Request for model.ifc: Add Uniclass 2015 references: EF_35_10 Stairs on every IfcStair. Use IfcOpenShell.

First a look at what the model holds.

```python
import ifcopenshell

model = ifcopenshell.open("model.ifc")
print(model.schema)
print("classifications:", [c.Name for c in model.by_type("IfcClassification")])
for ifc_class in ("IfcDoor", "IfcRoof", "IfcStair", "IfcWall", "IfcWindow"):
    print(ifc_class, len(model.by_type(ifc_class)))
```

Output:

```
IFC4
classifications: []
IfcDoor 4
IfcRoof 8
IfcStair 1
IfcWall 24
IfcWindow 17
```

```python
import ifcopenshell
import ifcopenshell.api.classification

model = ifcopenshell.open("model.ifc")

system = ifcopenshell.api.classification.add_classification(model, classification="Uniclass 2015")

codes = {
    "IfcStair": ("EF_35_10", "Stairs"),
}
for ifc_class, (code, name) in codes.items():
    products = model.by_type(ifc_class)
    ifcopenshell.api.classification.add_reference(
        model, products=products, classification=system, identification=code, name=name
    )
    print(code, len(products))

model.write("model_v2.ifc")
```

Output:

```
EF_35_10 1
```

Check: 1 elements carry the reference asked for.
